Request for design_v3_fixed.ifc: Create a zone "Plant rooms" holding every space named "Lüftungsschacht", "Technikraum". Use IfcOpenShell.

First a look at what the model holds.

```python
import ifcopenshell

model = ifcopenshell.open("design_v3_fixed.ifc")
print(model.schema)
seen = {}
for space in model.by_type("IfcSpace"):
    seen[space.LongName] = seen.get(space.LongName, 0) + 1
for name, count in sorted(seen.items(), key=str):
    print(count, "x", name)
print("zones:", [z.Name for z in model.by_type("IfcZone")][:20])
```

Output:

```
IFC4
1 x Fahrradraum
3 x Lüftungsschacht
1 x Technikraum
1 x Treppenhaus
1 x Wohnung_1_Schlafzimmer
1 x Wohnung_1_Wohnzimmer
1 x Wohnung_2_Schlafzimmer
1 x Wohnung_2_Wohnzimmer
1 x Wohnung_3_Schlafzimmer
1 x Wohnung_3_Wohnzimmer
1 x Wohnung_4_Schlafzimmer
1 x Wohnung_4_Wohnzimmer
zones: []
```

```python
import ifcopenshell
import ifcopenshell.api.group
import ifcopenshell.api.root

model = ifcopenshell.open("design_v3_fixed.ifc")

names = {"Lüftungsschacht", "Technikraum"}
spaces = [s for s in model.by_type("IfcSpace") if s.LongName in names]

zone = ifcopenshell.api.root.create_entity(model, ifc_class="IfcZone", name="Plant rooms")
ifcopenshell.api.group.assign_group(model, products=spaces, group=zone)
print(len(spaces), "spaces in", zone.Name)

model.write("design_v3_fixed_rev.ifc")
```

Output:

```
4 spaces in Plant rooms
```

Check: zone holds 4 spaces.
